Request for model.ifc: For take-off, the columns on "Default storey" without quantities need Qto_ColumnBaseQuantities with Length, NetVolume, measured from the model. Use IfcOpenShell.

First a look at what the model holds.

```python
import ifcopenshell
import ifcopenshell.util.element
import ifcopenshell.util.unit

model = ifcopenshell.open("model.ifc")
print(model.schema)
for unit_type in ("LENGTHUNIT", "AREAUNIT", "VOLUMEUNIT"):
    print(unit_type, ifcopenshell.util.unit.calculate_unit_scale(model, unit_type))
storey = next(s for s in model.by_type("IfcBuildingStorey") if s.Name == "Default storey")
columns = [e for e in ifcopenshell.util.element.get_decomposition(storey) if e.is_a("IfcColumn")]
for e in sorted(columns, key=lambda e: e.id()):
    print(e.id(), e.is_a(), e.Name, list(ifcopenshell.util.element.get_psets(e, qtos_only=True)), sep=" | ")
```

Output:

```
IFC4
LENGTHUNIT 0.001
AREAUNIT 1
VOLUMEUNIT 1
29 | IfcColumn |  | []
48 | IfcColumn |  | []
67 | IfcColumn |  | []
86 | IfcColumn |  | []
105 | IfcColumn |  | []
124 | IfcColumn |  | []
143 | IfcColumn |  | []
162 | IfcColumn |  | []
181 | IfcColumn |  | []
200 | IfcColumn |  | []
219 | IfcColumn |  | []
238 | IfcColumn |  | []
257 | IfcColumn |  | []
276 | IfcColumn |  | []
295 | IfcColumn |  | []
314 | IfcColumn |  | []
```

```python
import ifcopenshell
import ifcopenshell.api.pset
import ifcopenshell.geom
import ifcopenshell.util.element
import ifcopenshell.util.shape
import ifcopenshell.util.unit

model = ifcopenshell.open("model.ifc")
unit_scale = ifcopenshell.util.unit.calculate_unit_scale(model)
volume_scale = ifcopenshell.util.unit.calculate_unit_scale(model, "VOLUMEUNIT")
settings = ifcopenshell.geom.settings()

storey = next(s for s in model.by_type("IfcBuildingStorey") if s.Name == "Default storey")
columns = [e for e in ifcopenshell.util.element.get_decomposition(storey) if e.is_a("IfcColumn")]

for e in sorted(columns, key=lambda e: e.id()):
    if ifcopenshell.util.element.get_psets(e, qtos_only=True, should_inherit=False):
        continue
    # Geometry comes back in metres, in the element's own axes.
    shape = ifcopenshell.geom.create_shape(settings, e)
    values = {
        "Length": ifcopenshell.util.shape.get_z(shape.geometry) / unit_scale,
        "NetVolume": ifcopenshell.util.shape.get_volume(shape.geometry) / volume_scale,
    }
    qto = ifcopenshell.api.pset.add_qto(model, product=e, name="Qto_ColumnBaseQuantities")
    ifcopenshell.api.pset.edit_qto(model, qto=qto, properties=values)
    print(e.id(), {k: round(v, 3) for k, v in values.items()})

model.write("model_v2.ifc")
```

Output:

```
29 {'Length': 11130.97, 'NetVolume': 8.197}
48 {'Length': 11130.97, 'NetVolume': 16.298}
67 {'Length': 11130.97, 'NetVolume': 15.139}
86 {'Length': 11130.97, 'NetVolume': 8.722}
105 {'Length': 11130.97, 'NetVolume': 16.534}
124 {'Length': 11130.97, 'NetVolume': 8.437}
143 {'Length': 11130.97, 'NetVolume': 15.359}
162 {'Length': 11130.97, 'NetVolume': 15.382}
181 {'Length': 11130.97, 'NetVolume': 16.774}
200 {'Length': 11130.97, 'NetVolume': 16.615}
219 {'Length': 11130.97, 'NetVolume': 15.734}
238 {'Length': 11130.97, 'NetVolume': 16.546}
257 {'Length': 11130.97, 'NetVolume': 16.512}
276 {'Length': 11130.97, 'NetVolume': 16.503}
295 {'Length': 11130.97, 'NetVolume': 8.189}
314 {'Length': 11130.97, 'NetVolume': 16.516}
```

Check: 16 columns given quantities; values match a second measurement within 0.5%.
